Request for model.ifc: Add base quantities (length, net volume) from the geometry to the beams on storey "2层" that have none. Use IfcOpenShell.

First a look at what the model holds.

```python
import ifcopenshell
import ifcopenshell.util.element
import ifcopenshell.util.unit

model = ifcopenshell.open("model.ifc")
print(model.schema)
for unit_type in ("LENGTHUNIT", "AREAUNIT", "VOLUMEUNIT"):
    print(unit_type, ifcopenshell.util.unit.calculate_unit_scale(model, unit_type))
storey = next(s for s in model.by_type("IfcBuildingStorey") if s.Name == "2层")
beams = [e for e in ifcopenshell.util.element.get_decomposition(storey) if e.is_a("IfcBeam")]
for e in sorted(beams, key=lambda e: e.id()):
    print(e.id(), e.is_a(), e.Name, list(ifcopenshell.util.element.get_psets(e, qtos_only=True)), sep=" | ")
```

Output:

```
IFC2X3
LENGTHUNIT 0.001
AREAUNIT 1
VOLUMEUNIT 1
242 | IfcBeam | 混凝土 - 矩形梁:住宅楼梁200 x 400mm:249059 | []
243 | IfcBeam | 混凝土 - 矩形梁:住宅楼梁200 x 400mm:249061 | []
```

```python
import ifcopenshell
import ifcopenshell.api.pset
import ifcopenshell.geom
import ifcopenshell.util.element
import ifcopenshell.util.shape
import ifcopenshell.util.unit

model = ifcopenshell.open("model.ifc")
unit_scale = ifcopenshell.util.unit.calculate_unit_scale(model)
volume_scale = ifcopenshell.util.unit.calculate_unit_scale(model, "VOLUMEUNIT")
settings = ifcopenshell.geom.settings()

storey = next(s for s in model.by_type("IfcBuildingStorey") if s.Name == "2层")
beams = [e for e in ifcopenshell.util.element.get_decomposition(storey) if e.is_a("IfcBeam")]

for e in sorted(beams, key=lambda e: e.id()):
    if ifcopenshell.util.element.get_psets(e, qtos_only=True, should_inherit=False):
        continue
    # Geometry comes back in metres, in the element's own axes.
    shape = ifcopenshell.geom.create_shape(settings, e)
    values = {
        "Length": ifcopenshell.util.shape.get_max_xyz(shape.geometry) / unit_scale,
        "NetVolume": ifcopenshell.util.shape.get_volume(shape.geometry) / volume_scale,
    }
    qto = ifcopenshell.api.pset.add_qto(model, product=e, name="BaseQuantities")
    ifcopenshell.api.pset.edit_qto(model, qto=qto, properties=values)
    print(e.id(), {k: round(v, 3) for k, v in values.items()})

model.write("model-out.ifc")
```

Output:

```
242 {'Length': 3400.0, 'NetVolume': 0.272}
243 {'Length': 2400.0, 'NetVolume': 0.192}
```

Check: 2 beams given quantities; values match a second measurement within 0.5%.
